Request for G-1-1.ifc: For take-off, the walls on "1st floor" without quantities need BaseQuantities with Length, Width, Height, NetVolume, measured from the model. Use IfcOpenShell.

First a look at what the model holds.

```python
import ifcopenshell
import ifcopenshell.util.element
import ifcopenshell.util.unit

model = ifcopenshell.open("G-1-1.ifc")
print(model.schema)
for unit_type in ("LENGTHUNIT", "AREAUNIT", "VOLUMEUNIT"):
    print(unit_type, ifcopenshell.util.unit.calculate_unit_scale(model, unit_type))
storey = next(s for s in model.by_type("IfcBuildingStorey") if s.Name == "1st floor")
walls = [e for e in ifcopenshell.util.element.get_decomposition(storey) if e.is_a("IfcWall")]
for e in sorted(walls, key=lambda e: e.id()):
    print(e.id(), e.is_a(), e.Name, list(ifcopenshell.util.element.get_psets(e, qtos_only=True)), sep=" | ")
```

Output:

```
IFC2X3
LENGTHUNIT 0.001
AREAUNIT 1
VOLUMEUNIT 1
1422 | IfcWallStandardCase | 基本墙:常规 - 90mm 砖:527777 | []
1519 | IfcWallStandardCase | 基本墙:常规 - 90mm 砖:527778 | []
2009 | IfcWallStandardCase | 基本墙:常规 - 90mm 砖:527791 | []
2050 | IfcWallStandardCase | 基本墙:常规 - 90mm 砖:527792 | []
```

```python
import ifcopenshell
import ifcopenshell.api.pset
import ifcopenshell.geom
import ifcopenshell.util.element
import ifcopenshell.util.shape
import ifcopenshell.util.unit

model = ifcopenshell.open("G-1-1.ifc")
unit_scale = ifcopenshell.util.unit.calculate_unit_scale(model)
volume_scale = ifcopenshell.util.unit.calculate_unit_scale(model, "VOLUMEUNIT")
settings = ifcopenshell.geom.settings()

storey = next(s for s in model.by_type("IfcBuildingStorey") if s.Name == "1st floor")
walls = [e for e in ifcopenshell.util.element.get_decomposition(storey) if e.is_a("IfcWall")]

for e in sorted(walls, key=lambda e: e.id()):
    if ifcopenshell.util.element.get_psets(e, qtos_only=True, should_inherit=False):
        continue
    # Geometry comes back in metres, in the element's own axes.
    shape = ifcopenshell.geom.create_shape(settings, e)
    values = {
        "Length": ifcopenshell.util.shape.get_x(shape.geometry) / unit_scale,
        "Width": ifcopenshell.util.shape.get_y(shape.geometry) / unit_scale,
        "Height": ifcopenshell.util.shape.get_z(shape.geometry) / unit_scale,
        "NetVolume": ifcopenshell.util.shape.get_volume(shape.geometry) / volume_scale,
    }
    qto = ifcopenshell.api.pset.add_qto(model, product=e, name="BaseQuantities")
    ifcopenshell.api.pset.edit_qto(model, qto=qto, properties=values)
    print(e.id(), {k: round(v, 3) for k, v in values.items()})

model.write("G-1-1_rev.ifc")
```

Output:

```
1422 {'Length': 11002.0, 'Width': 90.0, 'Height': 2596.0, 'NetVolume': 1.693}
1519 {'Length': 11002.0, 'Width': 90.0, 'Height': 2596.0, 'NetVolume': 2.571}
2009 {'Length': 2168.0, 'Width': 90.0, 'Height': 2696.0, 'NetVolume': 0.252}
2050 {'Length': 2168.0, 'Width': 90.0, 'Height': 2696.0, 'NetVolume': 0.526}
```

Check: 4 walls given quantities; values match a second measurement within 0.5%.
